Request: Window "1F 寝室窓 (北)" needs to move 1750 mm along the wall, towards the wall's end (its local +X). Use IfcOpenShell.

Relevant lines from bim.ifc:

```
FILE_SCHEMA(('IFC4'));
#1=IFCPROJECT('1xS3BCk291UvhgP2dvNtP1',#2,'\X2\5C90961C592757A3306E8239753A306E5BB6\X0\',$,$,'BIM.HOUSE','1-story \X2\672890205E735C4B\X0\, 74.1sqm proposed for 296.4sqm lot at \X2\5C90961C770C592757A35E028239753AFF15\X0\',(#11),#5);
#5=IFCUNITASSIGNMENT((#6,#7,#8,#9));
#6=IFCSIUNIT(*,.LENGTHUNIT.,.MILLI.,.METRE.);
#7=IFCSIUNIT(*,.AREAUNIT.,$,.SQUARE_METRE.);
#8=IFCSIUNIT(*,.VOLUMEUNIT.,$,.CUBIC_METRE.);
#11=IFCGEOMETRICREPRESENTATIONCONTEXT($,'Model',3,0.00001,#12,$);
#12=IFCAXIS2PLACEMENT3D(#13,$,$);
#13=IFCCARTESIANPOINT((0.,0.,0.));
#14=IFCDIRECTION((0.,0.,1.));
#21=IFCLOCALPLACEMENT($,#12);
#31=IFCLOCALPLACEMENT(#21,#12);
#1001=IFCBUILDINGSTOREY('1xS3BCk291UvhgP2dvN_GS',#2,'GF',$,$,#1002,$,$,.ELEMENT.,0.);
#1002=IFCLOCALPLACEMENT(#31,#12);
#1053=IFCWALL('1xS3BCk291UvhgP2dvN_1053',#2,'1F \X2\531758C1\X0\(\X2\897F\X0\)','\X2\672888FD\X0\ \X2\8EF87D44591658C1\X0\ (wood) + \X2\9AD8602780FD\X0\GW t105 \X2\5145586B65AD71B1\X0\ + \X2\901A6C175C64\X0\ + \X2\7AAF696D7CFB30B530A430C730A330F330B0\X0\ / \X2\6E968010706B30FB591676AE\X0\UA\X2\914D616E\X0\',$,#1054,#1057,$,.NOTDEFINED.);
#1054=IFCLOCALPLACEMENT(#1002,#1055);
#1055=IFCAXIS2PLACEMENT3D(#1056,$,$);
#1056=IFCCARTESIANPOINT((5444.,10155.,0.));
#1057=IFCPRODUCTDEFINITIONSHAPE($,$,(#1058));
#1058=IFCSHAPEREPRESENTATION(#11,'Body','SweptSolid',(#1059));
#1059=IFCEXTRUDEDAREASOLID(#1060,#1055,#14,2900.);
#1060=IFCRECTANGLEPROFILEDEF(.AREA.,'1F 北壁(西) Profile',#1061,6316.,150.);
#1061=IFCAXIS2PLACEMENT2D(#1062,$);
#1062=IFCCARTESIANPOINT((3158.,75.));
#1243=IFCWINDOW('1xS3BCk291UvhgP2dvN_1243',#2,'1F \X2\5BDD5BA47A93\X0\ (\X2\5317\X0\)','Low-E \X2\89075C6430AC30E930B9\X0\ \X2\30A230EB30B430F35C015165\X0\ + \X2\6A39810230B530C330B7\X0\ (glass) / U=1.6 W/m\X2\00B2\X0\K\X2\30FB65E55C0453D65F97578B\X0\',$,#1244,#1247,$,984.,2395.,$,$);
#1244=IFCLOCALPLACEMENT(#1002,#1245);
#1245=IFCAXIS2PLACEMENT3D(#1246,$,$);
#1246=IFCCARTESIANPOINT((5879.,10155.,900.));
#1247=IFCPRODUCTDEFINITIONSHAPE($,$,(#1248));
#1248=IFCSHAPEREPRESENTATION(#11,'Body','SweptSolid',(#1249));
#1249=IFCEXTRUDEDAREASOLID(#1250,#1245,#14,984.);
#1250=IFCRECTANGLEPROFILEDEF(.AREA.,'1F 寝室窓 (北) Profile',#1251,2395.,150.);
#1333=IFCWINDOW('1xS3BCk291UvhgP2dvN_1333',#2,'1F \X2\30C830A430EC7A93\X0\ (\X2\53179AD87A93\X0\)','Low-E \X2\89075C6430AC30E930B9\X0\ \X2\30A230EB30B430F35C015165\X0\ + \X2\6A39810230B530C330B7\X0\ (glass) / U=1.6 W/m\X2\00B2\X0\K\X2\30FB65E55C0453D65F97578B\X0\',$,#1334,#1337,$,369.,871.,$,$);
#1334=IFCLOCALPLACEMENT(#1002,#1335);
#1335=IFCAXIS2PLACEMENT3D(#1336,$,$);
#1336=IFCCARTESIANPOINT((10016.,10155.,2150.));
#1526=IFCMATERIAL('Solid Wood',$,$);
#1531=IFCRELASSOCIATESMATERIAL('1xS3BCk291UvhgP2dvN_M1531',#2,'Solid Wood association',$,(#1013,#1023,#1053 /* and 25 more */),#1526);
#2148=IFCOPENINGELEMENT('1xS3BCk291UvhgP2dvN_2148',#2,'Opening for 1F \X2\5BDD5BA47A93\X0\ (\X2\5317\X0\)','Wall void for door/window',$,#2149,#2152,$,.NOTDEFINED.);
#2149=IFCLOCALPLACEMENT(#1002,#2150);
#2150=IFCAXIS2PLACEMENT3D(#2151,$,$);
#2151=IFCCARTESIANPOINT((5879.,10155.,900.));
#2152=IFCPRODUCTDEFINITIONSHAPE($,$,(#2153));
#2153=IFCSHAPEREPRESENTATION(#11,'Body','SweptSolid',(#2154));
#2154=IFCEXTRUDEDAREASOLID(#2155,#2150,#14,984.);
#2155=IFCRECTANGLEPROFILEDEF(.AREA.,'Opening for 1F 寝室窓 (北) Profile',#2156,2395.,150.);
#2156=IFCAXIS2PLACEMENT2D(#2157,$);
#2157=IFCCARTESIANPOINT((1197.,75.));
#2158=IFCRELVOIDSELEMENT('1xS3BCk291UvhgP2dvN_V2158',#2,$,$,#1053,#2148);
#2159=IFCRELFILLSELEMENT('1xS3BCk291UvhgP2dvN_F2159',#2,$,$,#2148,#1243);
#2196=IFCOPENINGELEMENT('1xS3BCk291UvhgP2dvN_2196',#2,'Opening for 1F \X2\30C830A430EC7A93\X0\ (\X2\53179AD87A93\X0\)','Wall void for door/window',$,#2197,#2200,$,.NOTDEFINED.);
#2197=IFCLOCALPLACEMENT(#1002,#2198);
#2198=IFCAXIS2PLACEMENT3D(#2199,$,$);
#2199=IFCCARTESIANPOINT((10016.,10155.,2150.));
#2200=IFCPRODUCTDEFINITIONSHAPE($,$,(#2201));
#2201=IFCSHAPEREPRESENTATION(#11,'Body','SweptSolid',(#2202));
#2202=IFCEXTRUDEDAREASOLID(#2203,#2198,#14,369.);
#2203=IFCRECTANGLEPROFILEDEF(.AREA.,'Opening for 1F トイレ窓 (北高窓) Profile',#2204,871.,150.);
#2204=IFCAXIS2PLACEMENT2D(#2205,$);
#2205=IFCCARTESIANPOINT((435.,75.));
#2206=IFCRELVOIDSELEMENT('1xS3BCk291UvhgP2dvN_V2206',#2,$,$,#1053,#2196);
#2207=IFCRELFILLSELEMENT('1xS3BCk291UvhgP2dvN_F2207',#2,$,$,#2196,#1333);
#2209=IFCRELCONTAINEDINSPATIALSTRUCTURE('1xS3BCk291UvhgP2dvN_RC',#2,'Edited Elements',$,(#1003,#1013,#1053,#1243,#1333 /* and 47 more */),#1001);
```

```python
import ifcopenshell
import ifcopenshell.api.geometry
import ifcopenshell.util.placement
import ifcopenshell.util.unit

model = ifcopenshell.open("bim.ifc")
unit_scale = ifcopenshell.util.unit.calculate_unit_scale(model)

window = model.by_id(1243)
opening = window.FillsVoids[0].RelatingOpeningElement
wall = opening.VoidsElements[0].RelatingBuildingElement

wall_matrix = ifcopenshell.util.placement.get_local_placement(wall.ObjectPlacement)
shift = wall_matrix[:3, 0] * 1.75 / unit_scale
before = ifcopenshell.util.placement.get_local_placement(window.ObjectPlacement)[:3, 3].copy()

# The window is not placed relative to its opening, so move both.
for product in (opening, window):
    matrix = ifcopenshell.util.placement.get_local_placement(product.ObjectPlacement)
    matrix[:3, 3] += shift
    ifcopenshell.api.geometry.edit_object_placement(model, product=product, matrix=matrix, is_si=False)

after = ifcopenshell.util.placement.get_local_placement(window.ObjectPlacement)[:3, 3]
print("window moved by", (after - before).round(3) + 0.0)

model.write("bim_edited.ifc")
```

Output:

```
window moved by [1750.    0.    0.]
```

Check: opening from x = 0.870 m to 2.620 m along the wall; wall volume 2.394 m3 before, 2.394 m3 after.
